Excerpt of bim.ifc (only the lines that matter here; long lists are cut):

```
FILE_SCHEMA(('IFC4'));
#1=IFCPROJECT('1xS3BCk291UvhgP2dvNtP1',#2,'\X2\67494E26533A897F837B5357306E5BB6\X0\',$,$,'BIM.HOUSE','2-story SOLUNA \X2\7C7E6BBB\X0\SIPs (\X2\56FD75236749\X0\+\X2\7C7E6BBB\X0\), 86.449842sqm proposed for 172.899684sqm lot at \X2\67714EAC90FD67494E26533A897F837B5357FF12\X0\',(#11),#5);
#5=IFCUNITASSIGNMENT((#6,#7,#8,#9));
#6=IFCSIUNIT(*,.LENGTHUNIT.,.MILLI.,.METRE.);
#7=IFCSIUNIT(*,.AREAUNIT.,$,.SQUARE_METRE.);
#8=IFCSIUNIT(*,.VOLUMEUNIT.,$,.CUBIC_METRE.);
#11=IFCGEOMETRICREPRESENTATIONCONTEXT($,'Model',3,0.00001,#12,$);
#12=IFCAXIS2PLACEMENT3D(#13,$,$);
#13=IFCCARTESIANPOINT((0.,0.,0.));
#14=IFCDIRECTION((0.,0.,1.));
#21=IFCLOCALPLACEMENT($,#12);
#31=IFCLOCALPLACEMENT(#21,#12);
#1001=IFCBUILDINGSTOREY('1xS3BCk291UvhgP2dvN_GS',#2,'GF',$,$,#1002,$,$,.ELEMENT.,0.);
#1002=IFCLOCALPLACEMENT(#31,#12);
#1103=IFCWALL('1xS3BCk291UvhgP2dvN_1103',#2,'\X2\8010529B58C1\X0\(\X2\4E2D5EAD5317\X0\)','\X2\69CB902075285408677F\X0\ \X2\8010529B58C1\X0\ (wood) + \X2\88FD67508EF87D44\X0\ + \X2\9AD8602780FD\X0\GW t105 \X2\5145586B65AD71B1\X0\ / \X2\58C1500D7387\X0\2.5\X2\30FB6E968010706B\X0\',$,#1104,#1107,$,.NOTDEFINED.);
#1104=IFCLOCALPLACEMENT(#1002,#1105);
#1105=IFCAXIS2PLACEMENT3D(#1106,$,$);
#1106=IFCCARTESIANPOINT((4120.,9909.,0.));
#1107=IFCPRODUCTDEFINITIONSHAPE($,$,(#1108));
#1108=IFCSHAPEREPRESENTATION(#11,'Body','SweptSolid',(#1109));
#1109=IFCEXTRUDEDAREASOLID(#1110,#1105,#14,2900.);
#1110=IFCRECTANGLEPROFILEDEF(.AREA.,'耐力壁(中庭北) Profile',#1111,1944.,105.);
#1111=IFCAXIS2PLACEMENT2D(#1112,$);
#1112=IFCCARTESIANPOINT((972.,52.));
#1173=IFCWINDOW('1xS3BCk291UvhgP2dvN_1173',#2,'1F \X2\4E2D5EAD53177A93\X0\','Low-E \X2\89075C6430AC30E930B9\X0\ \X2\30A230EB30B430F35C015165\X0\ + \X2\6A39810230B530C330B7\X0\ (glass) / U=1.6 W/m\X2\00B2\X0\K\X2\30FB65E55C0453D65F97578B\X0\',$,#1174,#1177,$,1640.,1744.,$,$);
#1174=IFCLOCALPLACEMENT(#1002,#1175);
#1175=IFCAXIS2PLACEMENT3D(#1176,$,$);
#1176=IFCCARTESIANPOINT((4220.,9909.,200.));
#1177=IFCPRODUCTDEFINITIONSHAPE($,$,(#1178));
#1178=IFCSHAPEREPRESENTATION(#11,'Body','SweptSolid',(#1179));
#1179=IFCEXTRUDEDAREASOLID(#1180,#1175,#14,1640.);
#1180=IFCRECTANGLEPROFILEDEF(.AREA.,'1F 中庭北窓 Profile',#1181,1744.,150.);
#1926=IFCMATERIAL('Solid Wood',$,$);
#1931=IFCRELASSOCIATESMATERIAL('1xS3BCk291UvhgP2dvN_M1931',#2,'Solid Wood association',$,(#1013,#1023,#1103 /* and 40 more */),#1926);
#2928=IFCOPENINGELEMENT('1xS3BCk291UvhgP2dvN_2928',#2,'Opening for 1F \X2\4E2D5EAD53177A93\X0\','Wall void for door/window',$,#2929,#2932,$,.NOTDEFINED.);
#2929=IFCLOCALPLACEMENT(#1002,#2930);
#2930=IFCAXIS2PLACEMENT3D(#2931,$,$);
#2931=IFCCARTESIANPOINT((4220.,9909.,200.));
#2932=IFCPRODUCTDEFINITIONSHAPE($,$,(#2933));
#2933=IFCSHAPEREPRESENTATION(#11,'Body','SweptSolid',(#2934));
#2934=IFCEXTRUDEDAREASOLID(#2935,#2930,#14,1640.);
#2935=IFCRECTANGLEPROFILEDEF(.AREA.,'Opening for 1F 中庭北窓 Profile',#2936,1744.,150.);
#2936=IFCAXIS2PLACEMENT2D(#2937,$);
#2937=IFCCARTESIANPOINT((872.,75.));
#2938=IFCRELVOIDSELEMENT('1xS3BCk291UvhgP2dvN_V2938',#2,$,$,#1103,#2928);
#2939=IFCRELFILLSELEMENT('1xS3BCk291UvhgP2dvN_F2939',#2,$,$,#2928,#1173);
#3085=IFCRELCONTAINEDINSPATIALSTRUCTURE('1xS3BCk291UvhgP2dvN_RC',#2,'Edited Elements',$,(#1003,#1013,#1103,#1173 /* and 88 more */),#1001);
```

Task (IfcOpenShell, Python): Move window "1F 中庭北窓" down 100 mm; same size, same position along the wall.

```python
import numpy as np
import ifcopenshell
import ifcopenshell.api.geometry
import ifcopenshell.util.placement
import ifcopenshell.util.unit

model = ifcopenshell.open("bim.ifc")
unit_scale = ifcopenshell.util.unit.calculate_unit_scale(model)

window = model.by_guid("1xS3BCk291UvhgP2dvN_1173")
opening = window.FillsVoids[0].RelatingOpeningElement
dz = -0.1 / unit_scale

shift = np.array([0.0, 0.0, dz])
# The window is not placed relative to its opening, so move both.
for product in (opening, window):
    matrix = ifcopenshell.util.placement.get_local_placement(product.ObjectPlacement)
    matrix[:3, 3] += shift
    ifcopenshell.api.geometry.edit_object_placement(model, product=product, matrix=matrix, is_si=False)

print(f"moved by {dz * unit_scale:+.3f} m")

model.write("bim_v2.ifc")
```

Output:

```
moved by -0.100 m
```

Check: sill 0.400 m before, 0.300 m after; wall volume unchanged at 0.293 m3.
